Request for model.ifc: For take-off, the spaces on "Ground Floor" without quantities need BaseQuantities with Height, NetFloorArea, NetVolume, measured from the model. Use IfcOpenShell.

First a look at what the model holds.

```python
import ifcopenshell
import ifcopenshell.util.element
import ifcopenshell.util.unit

model = ifcopenshell.open("model.ifc")
print(model.schema)
for unit_type in ("LENGTHUNIT", "AREAUNIT", "VOLUMEUNIT"):
    print(unit_type, ifcopenshell.util.unit.calculate_unit_scale(model, unit_type))
storey = next(s for s in model.by_type("IfcBuildingStorey") if s.Name == "Ground Floor")
spaces = [e for e in ifcopenshell.util.element.get_decomposition(storey) if e.is_a("IfcSpace")]
for e in sorted(spaces, key=lambda e: e.id()):
    print(e.id(), e.is_a(), e.Name, list(ifcopenshell.util.element.get_psets(e, qtos_only=True)), sep=" | ")
```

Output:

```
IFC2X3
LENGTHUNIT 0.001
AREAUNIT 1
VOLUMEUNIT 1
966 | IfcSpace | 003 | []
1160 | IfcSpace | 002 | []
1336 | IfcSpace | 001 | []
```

```python
import ifcopenshell
import ifcopenshell.api.pset
import ifcopenshell.geom
import ifcopenshell.util.element
import ifcopenshell.util.shape
import ifcopenshell.util.unit

model = ifcopenshell.open("model.ifc")
unit_scale = ifcopenshell.util.unit.calculate_unit_scale(model)
area_scale = ifcopenshell.util.unit.calculate_unit_scale(model, "AREAUNIT")
volume_scale = ifcopenshell.util.unit.calculate_unit_scale(model, "VOLUMEUNIT")
settings = ifcopenshell.geom.settings()

storey = next(s for s in model.by_type("IfcBuildingStorey") if s.Name == "Ground Floor")
spaces = [e for e in ifcopenshell.util.element.get_decomposition(storey) if e.is_a("IfcSpace")]

for e in sorted(spaces, key=lambda e: e.id()):
    if ifcopenshell.util.element.get_psets(e, qtos_only=True, should_inherit=False):
        continue
    # Geometry comes back in metres, in the element's own axes.
    shape = ifcopenshell.geom.create_shape(settings, e)
    values = {
        "Height": ifcopenshell.util.shape.get_z(shape.geometry) / unit_scale,
        "NetFloorArea": ifcopenshell.util.shape.get_footprint_area(shape.geometry) / area_scale,
        "NetVolume": ifcopenshell.util.shape.get_volume(shape.geometry) / volume_scale,
    }
    qto = ifcopenshell.api.pset.add_qto(model, product=e, name="BaseQuantities")
    ifcopenshell.api.pset.edit_qto(model, qto=qto, properties=values)
    print(e.id(), {k: round(v, 3) for k, v in values.items()})

model.write("model_v2.ifc")
```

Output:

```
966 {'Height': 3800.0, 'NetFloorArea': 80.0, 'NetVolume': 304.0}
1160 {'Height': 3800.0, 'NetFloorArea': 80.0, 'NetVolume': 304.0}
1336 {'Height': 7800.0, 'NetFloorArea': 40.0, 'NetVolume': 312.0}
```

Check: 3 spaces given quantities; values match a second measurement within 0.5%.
